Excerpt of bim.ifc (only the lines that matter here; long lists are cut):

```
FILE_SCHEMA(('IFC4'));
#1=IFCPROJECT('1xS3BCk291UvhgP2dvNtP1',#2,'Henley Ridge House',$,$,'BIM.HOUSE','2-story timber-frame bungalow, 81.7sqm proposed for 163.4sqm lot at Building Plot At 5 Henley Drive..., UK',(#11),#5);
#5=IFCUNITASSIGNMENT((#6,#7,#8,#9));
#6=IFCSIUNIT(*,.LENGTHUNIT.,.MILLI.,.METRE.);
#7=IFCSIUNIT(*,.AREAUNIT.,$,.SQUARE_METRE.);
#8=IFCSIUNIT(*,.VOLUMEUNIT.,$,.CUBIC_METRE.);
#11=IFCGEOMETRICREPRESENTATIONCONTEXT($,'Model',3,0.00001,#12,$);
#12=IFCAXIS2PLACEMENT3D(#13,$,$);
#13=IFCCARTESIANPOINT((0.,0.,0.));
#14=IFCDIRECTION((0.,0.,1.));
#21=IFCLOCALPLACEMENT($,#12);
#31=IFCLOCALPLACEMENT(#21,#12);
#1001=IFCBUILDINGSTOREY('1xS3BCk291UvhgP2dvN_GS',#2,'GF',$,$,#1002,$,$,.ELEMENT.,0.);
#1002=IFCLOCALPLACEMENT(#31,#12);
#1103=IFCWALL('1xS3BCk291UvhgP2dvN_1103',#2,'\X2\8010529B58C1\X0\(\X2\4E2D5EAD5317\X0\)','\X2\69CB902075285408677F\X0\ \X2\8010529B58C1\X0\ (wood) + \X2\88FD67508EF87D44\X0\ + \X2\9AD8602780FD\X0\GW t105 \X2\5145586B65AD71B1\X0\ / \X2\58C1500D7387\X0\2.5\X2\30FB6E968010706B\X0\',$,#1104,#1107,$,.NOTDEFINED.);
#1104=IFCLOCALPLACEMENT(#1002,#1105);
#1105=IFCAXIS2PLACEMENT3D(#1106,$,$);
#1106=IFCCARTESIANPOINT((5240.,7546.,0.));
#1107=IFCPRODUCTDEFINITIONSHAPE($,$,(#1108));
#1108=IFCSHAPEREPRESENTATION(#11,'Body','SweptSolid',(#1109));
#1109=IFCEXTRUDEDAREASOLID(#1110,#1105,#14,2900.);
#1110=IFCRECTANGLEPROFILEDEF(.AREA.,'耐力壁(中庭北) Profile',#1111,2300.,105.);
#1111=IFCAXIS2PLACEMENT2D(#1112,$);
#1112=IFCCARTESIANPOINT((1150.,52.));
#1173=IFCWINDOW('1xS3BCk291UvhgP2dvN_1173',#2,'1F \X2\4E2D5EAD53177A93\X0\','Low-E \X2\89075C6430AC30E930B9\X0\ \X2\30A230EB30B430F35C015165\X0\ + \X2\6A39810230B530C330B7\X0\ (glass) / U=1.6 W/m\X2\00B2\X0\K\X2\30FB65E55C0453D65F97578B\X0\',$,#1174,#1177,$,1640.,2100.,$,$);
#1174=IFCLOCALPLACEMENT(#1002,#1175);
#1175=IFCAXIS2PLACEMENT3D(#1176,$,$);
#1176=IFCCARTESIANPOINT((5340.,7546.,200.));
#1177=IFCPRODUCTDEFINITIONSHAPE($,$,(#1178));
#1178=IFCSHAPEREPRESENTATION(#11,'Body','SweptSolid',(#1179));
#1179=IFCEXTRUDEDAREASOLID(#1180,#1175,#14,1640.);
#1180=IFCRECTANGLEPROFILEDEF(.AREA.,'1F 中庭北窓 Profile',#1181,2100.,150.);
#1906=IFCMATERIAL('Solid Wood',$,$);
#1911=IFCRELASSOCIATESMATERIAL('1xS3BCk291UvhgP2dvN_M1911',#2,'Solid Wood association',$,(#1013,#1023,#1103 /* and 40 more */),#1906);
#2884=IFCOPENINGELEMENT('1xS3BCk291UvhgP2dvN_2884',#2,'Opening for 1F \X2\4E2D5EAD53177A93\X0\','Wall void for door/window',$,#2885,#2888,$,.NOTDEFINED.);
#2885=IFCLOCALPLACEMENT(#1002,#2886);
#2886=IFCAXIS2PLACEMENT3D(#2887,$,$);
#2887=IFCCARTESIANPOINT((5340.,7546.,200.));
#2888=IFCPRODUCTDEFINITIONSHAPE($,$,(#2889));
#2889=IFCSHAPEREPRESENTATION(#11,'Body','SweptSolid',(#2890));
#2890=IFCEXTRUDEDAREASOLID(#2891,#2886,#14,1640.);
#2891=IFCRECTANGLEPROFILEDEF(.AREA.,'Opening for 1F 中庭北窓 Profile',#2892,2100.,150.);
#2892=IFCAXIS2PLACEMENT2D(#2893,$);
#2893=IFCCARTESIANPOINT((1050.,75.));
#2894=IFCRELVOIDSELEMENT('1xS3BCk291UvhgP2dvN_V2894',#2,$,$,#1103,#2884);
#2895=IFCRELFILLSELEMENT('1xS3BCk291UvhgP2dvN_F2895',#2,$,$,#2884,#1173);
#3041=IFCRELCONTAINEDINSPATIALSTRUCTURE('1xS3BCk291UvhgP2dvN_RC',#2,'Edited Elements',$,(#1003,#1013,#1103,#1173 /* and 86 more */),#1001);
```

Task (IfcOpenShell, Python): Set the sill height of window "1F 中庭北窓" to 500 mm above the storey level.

```python
import numpy as np
import ifcopenshell
import ifcopenshell.api.geometry
import ifcopenshell.geom
import ifcopenshell.util.element
import ifcopenshell.util.placement
import ifcopenshell.util.shape
import ifcopenshell.util.unit

model = ifcopenshell.open("bim.ifc")
unit_scale = ifcopenshell.util.unit.calculate_unit_scale(model)

window = model.by_guid("1xS3BCk291UvhgP2dvN_1173")
opening = window.FillsVoids[0].RelatingOpeningElement
storey = ifcopenshell.util.element.get_container(window, ifc_class="IfcBuildingStorey")
level = ifcopenshell.util.placement.get_local_placement(storey.ObjectPlacement)[2, 3]

# The opening's origin need not be at the sill, so measure its lowest point.
shape = ifcopenshell.geom.create_shape(ifcopenshell.geom.settings(), opening)
bottom = ifcopenshell.util.shape.get_shape_bottom_elevation(shape, shape.geometry) / unit_scale
dz = level + 500.0 - bottom

shift = np.array([0.0, 0.0, dz])
# The window is not placed relative to its opening, so move both.
for product in (opening, window):
    matrix = ifcopenshell.util.placement.get_local_placement(product.ObjectPlacement)
    matrix[:3, 3] += shift
    ifcopenshell.api.geometry.edit_object_placement(model, product=product, matrix=matrix, is_si=False)

print(f"moved by {dz * unit_scale:+.3f} m")

model.write("bim_v2.ifc")
```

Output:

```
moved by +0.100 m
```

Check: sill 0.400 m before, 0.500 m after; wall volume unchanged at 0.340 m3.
